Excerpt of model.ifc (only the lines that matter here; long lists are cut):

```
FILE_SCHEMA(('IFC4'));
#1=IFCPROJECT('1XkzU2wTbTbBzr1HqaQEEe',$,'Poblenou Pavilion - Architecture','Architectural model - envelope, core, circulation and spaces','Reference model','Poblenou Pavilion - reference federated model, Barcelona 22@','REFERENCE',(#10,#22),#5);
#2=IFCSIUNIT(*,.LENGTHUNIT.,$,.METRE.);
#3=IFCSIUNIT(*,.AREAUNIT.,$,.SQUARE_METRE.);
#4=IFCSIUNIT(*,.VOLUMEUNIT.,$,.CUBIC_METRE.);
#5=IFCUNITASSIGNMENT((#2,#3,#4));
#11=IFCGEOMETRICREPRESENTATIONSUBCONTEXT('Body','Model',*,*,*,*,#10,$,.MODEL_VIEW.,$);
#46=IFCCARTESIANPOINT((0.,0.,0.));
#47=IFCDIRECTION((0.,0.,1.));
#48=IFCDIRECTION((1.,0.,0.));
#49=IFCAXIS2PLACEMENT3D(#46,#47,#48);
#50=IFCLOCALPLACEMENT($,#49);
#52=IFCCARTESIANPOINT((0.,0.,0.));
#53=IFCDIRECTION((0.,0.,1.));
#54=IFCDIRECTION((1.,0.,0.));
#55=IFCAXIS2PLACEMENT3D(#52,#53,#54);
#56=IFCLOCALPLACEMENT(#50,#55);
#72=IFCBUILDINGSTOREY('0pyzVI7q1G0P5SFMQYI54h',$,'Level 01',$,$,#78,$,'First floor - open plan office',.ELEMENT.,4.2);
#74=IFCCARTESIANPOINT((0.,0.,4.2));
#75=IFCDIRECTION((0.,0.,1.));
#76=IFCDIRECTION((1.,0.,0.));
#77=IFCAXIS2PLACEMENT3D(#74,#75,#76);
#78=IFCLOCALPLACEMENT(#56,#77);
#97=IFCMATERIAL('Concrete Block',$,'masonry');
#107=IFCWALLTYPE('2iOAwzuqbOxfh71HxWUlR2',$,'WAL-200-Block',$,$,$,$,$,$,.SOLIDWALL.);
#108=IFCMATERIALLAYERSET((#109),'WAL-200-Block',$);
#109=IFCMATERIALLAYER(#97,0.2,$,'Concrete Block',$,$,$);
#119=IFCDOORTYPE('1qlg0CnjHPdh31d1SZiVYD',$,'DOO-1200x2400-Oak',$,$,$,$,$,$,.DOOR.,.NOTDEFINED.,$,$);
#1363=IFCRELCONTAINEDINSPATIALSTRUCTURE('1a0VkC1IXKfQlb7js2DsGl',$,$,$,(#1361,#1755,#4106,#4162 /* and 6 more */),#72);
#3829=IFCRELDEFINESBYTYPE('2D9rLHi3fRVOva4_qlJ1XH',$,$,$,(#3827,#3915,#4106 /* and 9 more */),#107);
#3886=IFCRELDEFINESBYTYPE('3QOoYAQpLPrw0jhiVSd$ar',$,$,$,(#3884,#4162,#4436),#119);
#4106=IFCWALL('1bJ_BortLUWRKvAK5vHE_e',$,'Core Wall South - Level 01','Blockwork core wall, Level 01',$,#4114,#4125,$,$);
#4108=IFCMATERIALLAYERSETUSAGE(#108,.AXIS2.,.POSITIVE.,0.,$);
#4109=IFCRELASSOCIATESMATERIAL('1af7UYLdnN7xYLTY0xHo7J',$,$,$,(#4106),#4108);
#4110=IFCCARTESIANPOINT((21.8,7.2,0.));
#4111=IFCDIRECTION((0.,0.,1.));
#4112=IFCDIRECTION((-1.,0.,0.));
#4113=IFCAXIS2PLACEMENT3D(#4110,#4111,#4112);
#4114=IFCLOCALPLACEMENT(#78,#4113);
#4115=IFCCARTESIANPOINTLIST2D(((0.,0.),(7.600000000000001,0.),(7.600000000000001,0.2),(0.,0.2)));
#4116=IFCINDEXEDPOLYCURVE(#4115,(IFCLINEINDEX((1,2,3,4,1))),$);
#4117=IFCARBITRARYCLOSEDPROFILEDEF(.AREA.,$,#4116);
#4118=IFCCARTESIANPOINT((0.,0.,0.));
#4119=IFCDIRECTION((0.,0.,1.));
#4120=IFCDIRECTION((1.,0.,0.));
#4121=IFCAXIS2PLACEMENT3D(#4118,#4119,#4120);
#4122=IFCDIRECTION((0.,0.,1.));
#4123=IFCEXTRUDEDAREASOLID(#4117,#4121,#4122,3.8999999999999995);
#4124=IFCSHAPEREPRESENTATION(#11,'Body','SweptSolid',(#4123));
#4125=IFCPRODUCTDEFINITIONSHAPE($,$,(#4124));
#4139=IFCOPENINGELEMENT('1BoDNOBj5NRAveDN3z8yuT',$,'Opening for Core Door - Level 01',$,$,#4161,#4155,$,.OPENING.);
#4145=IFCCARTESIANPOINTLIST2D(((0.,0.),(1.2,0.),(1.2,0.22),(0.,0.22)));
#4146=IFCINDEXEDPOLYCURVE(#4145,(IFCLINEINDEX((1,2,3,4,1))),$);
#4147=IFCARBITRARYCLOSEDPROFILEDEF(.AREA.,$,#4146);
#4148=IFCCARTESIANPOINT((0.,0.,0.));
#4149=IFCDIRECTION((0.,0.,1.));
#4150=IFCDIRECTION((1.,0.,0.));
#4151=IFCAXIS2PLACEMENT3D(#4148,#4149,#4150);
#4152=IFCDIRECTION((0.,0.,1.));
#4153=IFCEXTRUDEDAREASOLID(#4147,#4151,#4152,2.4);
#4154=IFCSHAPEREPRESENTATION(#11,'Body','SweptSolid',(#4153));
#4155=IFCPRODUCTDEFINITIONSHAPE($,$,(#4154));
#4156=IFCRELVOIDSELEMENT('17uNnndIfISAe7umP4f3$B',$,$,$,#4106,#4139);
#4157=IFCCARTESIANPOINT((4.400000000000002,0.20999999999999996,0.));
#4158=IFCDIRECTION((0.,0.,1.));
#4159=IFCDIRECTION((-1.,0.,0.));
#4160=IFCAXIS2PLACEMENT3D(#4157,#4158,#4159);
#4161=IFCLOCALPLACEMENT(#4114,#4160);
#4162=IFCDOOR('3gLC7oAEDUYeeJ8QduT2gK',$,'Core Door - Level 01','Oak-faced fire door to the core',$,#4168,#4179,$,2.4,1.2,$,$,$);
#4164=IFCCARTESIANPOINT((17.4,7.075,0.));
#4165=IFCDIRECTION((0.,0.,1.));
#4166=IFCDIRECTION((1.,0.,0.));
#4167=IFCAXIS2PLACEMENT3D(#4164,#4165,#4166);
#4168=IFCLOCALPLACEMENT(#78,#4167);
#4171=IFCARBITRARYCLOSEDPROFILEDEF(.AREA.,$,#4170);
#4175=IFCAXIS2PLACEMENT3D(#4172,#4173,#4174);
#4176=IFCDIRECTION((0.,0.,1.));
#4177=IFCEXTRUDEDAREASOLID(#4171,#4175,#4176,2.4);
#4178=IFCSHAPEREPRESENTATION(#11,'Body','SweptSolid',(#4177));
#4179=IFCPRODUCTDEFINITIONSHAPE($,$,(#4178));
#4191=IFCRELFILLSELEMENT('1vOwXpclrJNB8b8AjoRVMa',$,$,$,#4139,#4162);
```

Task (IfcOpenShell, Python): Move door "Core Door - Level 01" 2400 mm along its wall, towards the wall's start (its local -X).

```python
import ifcopenshell
import ifcopenshell.api.geometry
import ifcopenshell.util.placement
import ifcopenshell.util.unit

model = ifcopenshell.open("model.ifc")
unit_scale = ifcopenshell.util.unit.calculate_unit_scale(model)

door = model.by_guid("3gLC7oAEDUYeeJ8QduT2gK")
opening = door.FillsVoids[0].RelatingOpeningElement
wall = opening.VoidsElements[0].RelatingBuildingElement

wall_matrix = ifcopenshell.util.placement.get_local_placement(wall.ObjectPlacement)
shift = wall_matrix[:3, 0] * -2.4 / unit_scale
before = ifcopenshell.util.placement.get_local_placement(door.ObjectPlacement)[:3, 3].copy()

# The door is not placed relative to its opening, so move both.
for product in (opening, door):
    matrix = ifcopenshell.util.placement.get_local_placement(product.ObjectPlacement)
    matrix[:3, 3] += shift
    ifcopenshell.api.geometry.edit_object_placement(model, product=product, matrix=matrix, is_si=False)

after = ifcopenshell.util.placement.get_local_placement(door.ObjectPlacement)[:3, 3]
print("door moved by", (after - before).round(3) + 0.0)

model.write("model_edited.ifc")
```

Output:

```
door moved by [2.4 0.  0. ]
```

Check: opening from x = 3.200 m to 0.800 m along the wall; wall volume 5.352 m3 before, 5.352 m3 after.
